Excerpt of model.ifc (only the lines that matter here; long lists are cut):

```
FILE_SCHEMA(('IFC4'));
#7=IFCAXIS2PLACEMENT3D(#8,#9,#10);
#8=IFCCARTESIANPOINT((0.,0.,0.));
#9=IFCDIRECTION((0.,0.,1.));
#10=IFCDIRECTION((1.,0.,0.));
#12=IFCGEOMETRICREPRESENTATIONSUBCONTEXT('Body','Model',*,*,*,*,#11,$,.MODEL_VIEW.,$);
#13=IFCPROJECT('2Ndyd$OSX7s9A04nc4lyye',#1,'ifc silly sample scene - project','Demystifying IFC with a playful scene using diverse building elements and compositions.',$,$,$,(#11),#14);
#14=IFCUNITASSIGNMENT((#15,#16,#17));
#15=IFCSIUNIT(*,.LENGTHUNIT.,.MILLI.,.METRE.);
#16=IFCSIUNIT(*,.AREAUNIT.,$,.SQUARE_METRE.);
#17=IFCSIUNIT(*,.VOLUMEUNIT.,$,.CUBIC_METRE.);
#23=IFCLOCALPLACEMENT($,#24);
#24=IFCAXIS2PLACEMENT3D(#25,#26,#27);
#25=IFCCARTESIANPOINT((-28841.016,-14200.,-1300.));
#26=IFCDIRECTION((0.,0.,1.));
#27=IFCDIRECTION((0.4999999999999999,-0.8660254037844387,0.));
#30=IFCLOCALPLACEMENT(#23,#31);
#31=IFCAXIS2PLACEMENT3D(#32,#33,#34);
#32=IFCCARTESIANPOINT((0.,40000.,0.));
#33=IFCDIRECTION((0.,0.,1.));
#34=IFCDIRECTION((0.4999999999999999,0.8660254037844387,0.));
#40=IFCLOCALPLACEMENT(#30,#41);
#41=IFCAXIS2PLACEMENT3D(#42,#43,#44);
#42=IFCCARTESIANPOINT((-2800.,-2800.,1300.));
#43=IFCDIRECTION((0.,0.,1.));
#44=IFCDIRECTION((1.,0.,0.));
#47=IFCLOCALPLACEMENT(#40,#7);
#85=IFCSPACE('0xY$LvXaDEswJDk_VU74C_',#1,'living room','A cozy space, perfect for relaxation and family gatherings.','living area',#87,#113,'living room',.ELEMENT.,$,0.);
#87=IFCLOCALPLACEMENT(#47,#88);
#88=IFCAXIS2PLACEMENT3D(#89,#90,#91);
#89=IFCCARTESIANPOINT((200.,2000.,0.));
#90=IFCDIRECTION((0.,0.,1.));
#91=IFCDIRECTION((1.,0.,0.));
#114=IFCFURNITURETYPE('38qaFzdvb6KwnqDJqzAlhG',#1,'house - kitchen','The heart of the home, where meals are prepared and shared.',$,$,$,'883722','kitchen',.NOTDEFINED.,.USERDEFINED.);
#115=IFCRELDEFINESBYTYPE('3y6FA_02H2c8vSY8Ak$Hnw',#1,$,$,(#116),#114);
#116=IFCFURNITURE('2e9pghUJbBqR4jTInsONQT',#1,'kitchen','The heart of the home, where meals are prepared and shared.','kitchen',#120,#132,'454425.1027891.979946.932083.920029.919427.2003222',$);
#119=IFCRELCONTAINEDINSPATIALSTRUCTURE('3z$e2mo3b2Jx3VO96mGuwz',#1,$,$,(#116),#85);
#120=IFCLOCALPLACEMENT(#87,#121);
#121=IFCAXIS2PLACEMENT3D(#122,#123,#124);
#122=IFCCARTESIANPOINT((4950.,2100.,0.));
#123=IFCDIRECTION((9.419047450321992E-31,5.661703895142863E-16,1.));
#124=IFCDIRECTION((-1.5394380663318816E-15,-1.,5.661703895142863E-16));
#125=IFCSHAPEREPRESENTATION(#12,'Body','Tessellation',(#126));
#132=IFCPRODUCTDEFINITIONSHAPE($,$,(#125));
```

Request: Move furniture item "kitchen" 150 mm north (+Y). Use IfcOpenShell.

```python
import ifcopenshell
import ifcopenshell.api.geometry
import ifcopenshell.util.placement

model = ifcopenshell.open("model.ifc")

item = model.by_guid("2e9pghUJbBqR4jTInsONQT")
matrix = ifcopenshell.util.placement.get_local_placement(item.ObjectPlacement)
matrix[1, 3] += 150.0
ifcopenshell.api.geometry.edit_object_placement(model, product=item, matrix=matrix, is_si=False)

print(ifcopenshell.util.placement.get_local_placement(item.ObjectPlacement).round(3) + 0.0)

model.write("model_v2.ifc")
```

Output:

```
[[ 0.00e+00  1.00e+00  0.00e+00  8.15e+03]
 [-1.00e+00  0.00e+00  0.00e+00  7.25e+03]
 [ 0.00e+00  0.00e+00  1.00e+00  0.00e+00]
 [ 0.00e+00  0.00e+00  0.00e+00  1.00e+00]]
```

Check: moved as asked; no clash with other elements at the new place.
